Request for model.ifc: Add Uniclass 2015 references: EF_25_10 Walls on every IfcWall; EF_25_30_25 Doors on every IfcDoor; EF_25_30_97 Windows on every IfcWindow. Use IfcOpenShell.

First a look at what the model holds.

```python
import ifcopenshell

model = ifcopenshell.open("model.ifc")
print(model.schema)
print("classifications:", [c.Name for c in model.by_type("IfcClassification")])
for ifc_class in ("IfcDoor", "IfcRoof", "IfcStair", "IfcWall", "IfcWindow"):
    print(ifc_class, len(model.by_type(ifc_class)))
```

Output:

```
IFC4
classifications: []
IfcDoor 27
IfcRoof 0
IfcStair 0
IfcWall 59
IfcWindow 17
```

```python
import ifcopenshell
import ifcopenshell.api.classification

model = ifcopenshell.open("model.ifc")

system = ifcopenshell.api.classification.add_classification(model, classification="Uniclass 2015")

codes = {
    "IfcWall": ("EF_25_10", "Walls"),
    "IfcDoor": ("EF_25_30_25", "Doors"),
    "IfcWindow": ("EF_25_30_97", "Windows"),
}
for ifc_class, (code, name) in codes.items():
    products = model.by_type(ifc_class)
    ifcopenshell.api.classification.add_reference(
        model, products=products, classification=system, identification=code, name=name
    )
    print(code, len(products))

model.write("model_edited.ifc")
```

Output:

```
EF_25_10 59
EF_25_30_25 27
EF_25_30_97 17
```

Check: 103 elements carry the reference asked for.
